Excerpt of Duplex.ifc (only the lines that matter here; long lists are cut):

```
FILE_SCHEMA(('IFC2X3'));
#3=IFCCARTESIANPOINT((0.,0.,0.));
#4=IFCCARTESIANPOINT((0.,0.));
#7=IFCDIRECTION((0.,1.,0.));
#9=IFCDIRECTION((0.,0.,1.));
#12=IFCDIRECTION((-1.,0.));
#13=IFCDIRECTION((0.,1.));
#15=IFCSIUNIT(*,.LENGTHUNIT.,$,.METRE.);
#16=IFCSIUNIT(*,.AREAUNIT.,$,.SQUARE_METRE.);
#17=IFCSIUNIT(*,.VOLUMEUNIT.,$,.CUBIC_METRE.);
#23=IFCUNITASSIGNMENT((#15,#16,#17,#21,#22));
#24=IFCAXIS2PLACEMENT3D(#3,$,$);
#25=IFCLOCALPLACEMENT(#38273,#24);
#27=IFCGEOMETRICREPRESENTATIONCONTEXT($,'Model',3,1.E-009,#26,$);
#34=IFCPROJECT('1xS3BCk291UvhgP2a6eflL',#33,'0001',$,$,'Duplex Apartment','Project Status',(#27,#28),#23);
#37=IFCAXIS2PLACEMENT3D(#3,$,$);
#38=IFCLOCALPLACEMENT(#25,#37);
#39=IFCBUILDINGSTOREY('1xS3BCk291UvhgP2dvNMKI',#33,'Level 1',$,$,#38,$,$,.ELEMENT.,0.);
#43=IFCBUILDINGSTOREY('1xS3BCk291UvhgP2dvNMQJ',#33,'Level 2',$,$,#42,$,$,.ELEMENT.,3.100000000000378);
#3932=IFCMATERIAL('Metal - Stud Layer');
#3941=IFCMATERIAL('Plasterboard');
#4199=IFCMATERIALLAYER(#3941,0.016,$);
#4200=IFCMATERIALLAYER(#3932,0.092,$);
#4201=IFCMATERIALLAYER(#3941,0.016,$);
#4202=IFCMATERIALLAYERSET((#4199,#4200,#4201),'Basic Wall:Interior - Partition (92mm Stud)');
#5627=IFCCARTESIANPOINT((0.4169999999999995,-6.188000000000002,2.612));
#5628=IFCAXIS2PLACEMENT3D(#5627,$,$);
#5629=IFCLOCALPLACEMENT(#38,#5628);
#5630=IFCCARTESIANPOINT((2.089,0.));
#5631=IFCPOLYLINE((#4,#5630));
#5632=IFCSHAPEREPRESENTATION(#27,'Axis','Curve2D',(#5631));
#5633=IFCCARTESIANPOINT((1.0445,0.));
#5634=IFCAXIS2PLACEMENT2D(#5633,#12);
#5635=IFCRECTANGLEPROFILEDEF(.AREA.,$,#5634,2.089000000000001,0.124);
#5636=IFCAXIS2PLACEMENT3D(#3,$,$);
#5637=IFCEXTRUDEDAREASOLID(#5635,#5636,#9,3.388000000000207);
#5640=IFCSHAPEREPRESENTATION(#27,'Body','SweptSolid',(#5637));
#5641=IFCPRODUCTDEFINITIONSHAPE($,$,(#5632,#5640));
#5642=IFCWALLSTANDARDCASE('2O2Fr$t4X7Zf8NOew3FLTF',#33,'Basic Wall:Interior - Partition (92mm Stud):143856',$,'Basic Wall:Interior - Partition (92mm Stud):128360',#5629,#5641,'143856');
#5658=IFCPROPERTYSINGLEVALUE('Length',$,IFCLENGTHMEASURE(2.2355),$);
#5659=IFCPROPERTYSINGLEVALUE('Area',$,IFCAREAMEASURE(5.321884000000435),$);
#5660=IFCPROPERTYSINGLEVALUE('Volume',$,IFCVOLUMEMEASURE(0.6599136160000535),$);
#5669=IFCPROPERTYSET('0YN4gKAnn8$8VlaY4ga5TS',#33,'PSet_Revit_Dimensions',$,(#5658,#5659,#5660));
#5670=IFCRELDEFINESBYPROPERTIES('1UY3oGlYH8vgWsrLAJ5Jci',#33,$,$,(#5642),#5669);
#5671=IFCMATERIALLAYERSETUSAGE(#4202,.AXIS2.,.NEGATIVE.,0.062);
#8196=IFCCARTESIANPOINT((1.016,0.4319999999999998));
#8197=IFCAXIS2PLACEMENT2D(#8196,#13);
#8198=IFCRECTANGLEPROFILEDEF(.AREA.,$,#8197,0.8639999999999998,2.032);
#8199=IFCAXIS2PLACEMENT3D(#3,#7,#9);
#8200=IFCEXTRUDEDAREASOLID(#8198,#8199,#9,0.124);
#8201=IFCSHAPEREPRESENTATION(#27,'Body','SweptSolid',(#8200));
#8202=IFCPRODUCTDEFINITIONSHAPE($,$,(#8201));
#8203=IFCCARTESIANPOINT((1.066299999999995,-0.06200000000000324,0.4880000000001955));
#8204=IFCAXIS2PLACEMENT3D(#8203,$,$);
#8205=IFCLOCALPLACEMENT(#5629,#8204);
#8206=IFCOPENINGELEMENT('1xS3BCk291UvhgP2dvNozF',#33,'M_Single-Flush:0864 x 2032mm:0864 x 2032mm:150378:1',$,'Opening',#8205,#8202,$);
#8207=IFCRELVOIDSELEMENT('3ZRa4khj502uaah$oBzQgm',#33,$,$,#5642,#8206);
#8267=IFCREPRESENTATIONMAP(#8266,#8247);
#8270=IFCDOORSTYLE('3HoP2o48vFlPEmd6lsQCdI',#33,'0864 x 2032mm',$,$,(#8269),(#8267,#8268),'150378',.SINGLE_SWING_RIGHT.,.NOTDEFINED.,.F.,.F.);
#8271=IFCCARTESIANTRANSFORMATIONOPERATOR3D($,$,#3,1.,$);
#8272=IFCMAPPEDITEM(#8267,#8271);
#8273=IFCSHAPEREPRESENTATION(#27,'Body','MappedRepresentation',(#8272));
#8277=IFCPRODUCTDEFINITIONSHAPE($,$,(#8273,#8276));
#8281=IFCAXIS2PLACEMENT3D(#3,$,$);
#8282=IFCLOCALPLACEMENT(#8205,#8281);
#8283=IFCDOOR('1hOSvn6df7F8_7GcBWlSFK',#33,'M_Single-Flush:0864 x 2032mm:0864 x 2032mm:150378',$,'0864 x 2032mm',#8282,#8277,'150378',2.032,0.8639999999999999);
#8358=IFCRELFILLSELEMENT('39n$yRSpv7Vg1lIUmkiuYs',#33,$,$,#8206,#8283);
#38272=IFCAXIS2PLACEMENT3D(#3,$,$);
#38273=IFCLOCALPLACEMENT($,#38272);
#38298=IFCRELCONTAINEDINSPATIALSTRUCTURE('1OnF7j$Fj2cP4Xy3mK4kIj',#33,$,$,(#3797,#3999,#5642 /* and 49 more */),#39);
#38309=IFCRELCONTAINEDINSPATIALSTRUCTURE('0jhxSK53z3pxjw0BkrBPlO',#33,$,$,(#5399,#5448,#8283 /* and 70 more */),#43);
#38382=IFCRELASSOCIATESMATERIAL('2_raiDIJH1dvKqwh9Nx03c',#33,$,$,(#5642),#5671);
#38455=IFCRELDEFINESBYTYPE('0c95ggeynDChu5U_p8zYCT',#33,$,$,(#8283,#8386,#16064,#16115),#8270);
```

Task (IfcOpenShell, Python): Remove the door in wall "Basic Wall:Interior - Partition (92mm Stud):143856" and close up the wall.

```python
import ifcopenshell
import ifcopenshell.api.feature
import ifcopenshell.api.pset
import ifcopenshell.api.root
import ifcopenshell.geom
import ifcopenshell.util.element
import ifcopenshell.util.shape
import ifcopenshell.util.unit

model = ifcopenshell.open("Duplex.ifc")
area_scale = ifcopenshell.util.unit.calculate_unit_scale(model, "AREAUNIT")
volume_scale = ifcopenshell.util.unit.calculate_unit_scale(model, "VOLUMEUNIT")
settings = ifcopenshell.geom.settings()


def volume(element):
    """Net volume in cubic metres, openings subtracted."""
    shape = ifcopenshell.geom.create_shape(settings, element)
    return ifcopenshell.util.shape.get_volume(shape.geometry)


door = model.by_guid("1hOSvn6df7F8_7GcBWlSFK")
opening = door.FillsVoids[0].RelatingOpeningElement
wall = opening.VoidsElements[0].RelatingBuildingElement
before = volume(wall)

ifcopenshell.api.root.remove_product(model, product=door)
ifcopenshell.api.feature.remove_feature(model, feature=opening)

after = volume(wall)
thickness = 0.124  # wall thickness in metres

# Update the wall's stored quantities.
pset = model.by_id(ifcopenshell.util.element.get_pset(wall, "PSet_Revit_Dimensions", should_inherit=False)["id"])
ifcopenshell.api.pset.edit_pset(model, pset=pset, properties={
    "Area": model.create_entity("IfcAreaMeasure", after / thickness / area_scale),
    "Volume": model.create_entity("IfcVolumeMeasure", after / volume_scale),
})

print(f"wall volume {before:.3f} -> {after:.3f} m3")

model.write("Duplex_edited.ifc")
```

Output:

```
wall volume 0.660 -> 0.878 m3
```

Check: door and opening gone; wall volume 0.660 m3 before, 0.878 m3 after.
